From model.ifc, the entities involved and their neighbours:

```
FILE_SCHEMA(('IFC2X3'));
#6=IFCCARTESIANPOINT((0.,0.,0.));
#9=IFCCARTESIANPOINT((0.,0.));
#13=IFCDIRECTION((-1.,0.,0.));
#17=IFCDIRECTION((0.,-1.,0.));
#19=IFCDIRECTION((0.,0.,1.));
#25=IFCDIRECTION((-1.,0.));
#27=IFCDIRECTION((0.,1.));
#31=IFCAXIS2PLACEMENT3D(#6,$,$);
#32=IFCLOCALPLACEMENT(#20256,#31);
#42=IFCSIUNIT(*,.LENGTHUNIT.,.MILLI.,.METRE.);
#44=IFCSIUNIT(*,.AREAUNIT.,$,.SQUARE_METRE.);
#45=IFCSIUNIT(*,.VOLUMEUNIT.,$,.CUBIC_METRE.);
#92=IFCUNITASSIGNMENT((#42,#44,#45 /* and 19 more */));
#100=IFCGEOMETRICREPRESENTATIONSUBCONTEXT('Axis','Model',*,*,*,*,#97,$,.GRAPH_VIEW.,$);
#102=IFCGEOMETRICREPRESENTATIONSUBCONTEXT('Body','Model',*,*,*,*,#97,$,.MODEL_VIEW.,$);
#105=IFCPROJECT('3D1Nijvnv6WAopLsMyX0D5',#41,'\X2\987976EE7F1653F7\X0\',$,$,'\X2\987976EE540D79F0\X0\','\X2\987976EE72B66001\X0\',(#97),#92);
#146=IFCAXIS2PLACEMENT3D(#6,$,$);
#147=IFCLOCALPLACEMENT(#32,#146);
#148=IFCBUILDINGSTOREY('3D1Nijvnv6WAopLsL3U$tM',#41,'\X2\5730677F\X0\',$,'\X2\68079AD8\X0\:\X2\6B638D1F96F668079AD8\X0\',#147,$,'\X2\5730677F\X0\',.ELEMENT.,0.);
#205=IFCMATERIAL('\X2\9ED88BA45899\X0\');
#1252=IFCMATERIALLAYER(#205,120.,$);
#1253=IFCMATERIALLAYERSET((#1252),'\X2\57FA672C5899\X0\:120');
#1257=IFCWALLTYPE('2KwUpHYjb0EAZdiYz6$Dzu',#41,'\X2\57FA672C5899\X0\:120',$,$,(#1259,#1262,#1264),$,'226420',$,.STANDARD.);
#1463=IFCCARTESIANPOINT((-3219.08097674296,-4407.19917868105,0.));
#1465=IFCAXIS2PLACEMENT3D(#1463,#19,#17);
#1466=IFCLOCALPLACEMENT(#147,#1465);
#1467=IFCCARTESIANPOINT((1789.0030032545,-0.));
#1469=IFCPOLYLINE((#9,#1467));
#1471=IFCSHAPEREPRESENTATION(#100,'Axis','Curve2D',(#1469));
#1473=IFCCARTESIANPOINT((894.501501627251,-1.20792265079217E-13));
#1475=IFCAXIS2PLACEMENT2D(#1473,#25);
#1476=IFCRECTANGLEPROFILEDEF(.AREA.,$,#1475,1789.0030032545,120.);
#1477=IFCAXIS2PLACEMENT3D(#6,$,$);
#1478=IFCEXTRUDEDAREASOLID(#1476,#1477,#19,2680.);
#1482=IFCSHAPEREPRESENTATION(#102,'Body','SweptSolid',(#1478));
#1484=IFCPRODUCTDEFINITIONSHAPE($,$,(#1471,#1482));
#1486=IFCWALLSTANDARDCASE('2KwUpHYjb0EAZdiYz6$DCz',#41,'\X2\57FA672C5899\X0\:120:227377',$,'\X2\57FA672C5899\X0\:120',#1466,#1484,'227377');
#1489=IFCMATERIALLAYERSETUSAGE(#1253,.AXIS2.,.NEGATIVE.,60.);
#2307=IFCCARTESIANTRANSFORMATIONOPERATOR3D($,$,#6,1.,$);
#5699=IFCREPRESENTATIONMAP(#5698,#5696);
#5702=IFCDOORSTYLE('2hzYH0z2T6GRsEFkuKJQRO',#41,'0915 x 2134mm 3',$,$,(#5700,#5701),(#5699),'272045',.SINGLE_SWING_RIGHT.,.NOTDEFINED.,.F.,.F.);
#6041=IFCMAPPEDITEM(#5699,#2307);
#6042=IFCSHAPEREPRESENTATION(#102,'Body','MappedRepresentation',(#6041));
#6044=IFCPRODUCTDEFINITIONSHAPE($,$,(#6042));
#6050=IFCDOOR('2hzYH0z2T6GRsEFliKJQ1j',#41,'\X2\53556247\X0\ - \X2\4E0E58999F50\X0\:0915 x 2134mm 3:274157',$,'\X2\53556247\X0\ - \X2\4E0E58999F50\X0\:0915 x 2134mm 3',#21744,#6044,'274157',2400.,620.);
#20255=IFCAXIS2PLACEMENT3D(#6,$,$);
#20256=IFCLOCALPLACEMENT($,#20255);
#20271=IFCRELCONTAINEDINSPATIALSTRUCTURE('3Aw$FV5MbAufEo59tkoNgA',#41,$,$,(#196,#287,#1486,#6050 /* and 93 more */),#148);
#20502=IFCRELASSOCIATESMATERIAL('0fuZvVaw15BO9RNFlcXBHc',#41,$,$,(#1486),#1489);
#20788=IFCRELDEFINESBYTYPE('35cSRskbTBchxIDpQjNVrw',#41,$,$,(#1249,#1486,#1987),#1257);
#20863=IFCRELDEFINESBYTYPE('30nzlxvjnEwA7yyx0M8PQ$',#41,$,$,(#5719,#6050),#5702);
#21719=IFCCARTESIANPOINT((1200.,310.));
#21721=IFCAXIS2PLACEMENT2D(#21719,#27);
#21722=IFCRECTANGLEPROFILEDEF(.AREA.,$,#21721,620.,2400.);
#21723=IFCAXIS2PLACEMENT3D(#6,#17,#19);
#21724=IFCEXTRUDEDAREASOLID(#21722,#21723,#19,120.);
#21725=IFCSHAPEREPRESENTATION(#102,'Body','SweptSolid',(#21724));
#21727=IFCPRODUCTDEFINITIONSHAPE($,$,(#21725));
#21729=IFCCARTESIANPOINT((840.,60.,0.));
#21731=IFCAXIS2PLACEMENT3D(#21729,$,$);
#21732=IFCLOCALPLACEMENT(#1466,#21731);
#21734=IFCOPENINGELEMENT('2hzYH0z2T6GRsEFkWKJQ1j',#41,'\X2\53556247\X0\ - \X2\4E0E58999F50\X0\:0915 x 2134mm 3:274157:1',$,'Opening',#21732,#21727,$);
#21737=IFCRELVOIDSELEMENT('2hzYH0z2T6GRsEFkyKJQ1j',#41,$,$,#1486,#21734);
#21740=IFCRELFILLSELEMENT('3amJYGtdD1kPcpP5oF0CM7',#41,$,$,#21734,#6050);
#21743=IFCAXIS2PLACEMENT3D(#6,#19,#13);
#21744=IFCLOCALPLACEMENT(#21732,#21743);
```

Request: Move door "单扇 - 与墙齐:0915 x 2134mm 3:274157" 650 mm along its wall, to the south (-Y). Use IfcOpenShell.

```python
import ifcopenshell
import ifcopenshell.api.geometry
import ifcopenshell.util.placement
import ifcopenshell.util.unit

model = ifcopenshell.open("model.ifc")
unit_scale = ifcopenshell.util.unit.calculate_unit_scale(model)

door = model.by_guid("2hzYH0z2T6GRsEFliKJQ1j")
opening = door.FillsVoids[0].RelatingOpeningElement
wall = opening.VoidsElements[0].RelatingBuildingElement

wall_matrix = ifcopenshell.util.placement.get_local_placement(wall.ObjectPlacement)
shift = wall_matrix[:3, 0] * 0.65 / unit_scale
before = ifcopenshell.util.placement.get_local_placement(door.ObjectPlacement)[:3, 3].copy()

# The door is placed relative to its opening, so it follows when the opening moves.
matrix = ifcopenshell.util.placement.get_local_placement(opening.ObjectPlacement)
matrix[:3, 3] += shift
ifcopenshell.api.geometry.edit_object_placement(
    model, product=opening, matrix=matrix, is_si=False, should_transform_children=True
)

after = ifcopenshell.util.placement.get_local_placement(door.ObjectPlacement)[:3, 3]
print("door moved by", (after - before).round(3) + 0.0)

model.write("model_updated.ifc")
```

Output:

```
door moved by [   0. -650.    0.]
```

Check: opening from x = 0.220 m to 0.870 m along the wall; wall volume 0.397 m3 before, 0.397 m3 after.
